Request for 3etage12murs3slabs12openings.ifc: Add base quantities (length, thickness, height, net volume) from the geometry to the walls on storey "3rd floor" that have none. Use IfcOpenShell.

First a look at what the model holds.

```python
import ifcopenshell
import ifcopenshell.util.element
import ifcopenshell.util.unit

model = ifcopenshell.open("3etage12murs3slabs12openings.ifc")
print(model.schema)
for unit_type in ("LENGTHUNIT", "AREAUNIT", "VOLUMEUNIT"):
    print(unit_type, ifcopenshell.util.unit.calculate_unit_scale(model, unit_type))
storey = next(s for s in model.by_type("IfcBuildingStorey") if s.Name == "3rd floor")
walls = [e for e in ifcopenshell.util.element.get_decomposition(storey) if e.is_a("IfcWall")]
for e in sorted(walls, key=lambda e: e.id()):
    print(e.id(), e.is_a(), e.Name, list(ifcopenshell.util.element.get_psets(e, qtos_only=True)), sep=" | ")
```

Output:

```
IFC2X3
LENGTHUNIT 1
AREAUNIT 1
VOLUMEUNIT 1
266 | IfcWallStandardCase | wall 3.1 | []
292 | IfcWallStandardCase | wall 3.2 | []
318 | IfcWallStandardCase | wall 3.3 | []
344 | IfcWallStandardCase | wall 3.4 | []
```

```python
import ifcopenshell
import ifcopenshell.api.pset
import ifcopenshell.geom
import ifcopenshell.util.element
import ifcopenshell.util.shape
import ifcopenshell.util.unit

model = ifcopenshell.open("3etage12murs3slabs12openings.ifc")
unit_scale = ifcopenshell.util.unit.calculate_unit_scale(model)
volume_scale = ifcopenshell.util.unit.calculate_unit_scale(model, "VOLUMEUNIT")
settings = ifcopenshell.geom.settings()

storey = next(s for s in model.by_type("IfcBuildingStorey") if s.Name == "3rd floor")
walls = [e for e in ifcopenshell.util.element.get_decomposition(storey) if e.is_a("IfcWall")]

for e in sorted(walls, key=lambda e: e.id()):
    if ifcopenshell.util.element.get_psets(e, qtos_only=True, should_inherit=False):
        continue
    # Geometry comes back in metres, in the element's own axes.
    shape = ifcopenshell.geom.create_shape(settings, e)
    values = {
        "Length": ifcopenshell.util.shape.get_x(shape.geometry) / unit_scale,
        "Width": ifcopenshell.util.shape.get_y(shape.geometry) / unit_scale,
        "Height": ifcopenshell.util.shape.get_z(shape.geometry) / unit_scale,
        "NetVolume": ifcopenshell.util.shape.get_volume(shape.geometry) / volume_scale,
    }
    qto = ifcopenshell.api.pset.add_qto(model, product=e, name="BaseQuantities")
    ifcopenshell.api.pset.edit_qto(model, qto=qto, properties=values)
    print(e.id(), {k: round(v, 3) for k, v in values.items()})

model.write("3etage12murs3slabs12openings_v2.ifc")
```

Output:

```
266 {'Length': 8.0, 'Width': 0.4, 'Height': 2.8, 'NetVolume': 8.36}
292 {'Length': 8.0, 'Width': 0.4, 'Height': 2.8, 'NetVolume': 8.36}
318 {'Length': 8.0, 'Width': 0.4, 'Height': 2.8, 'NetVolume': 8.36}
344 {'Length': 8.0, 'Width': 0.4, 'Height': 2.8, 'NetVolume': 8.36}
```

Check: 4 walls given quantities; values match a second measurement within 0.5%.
